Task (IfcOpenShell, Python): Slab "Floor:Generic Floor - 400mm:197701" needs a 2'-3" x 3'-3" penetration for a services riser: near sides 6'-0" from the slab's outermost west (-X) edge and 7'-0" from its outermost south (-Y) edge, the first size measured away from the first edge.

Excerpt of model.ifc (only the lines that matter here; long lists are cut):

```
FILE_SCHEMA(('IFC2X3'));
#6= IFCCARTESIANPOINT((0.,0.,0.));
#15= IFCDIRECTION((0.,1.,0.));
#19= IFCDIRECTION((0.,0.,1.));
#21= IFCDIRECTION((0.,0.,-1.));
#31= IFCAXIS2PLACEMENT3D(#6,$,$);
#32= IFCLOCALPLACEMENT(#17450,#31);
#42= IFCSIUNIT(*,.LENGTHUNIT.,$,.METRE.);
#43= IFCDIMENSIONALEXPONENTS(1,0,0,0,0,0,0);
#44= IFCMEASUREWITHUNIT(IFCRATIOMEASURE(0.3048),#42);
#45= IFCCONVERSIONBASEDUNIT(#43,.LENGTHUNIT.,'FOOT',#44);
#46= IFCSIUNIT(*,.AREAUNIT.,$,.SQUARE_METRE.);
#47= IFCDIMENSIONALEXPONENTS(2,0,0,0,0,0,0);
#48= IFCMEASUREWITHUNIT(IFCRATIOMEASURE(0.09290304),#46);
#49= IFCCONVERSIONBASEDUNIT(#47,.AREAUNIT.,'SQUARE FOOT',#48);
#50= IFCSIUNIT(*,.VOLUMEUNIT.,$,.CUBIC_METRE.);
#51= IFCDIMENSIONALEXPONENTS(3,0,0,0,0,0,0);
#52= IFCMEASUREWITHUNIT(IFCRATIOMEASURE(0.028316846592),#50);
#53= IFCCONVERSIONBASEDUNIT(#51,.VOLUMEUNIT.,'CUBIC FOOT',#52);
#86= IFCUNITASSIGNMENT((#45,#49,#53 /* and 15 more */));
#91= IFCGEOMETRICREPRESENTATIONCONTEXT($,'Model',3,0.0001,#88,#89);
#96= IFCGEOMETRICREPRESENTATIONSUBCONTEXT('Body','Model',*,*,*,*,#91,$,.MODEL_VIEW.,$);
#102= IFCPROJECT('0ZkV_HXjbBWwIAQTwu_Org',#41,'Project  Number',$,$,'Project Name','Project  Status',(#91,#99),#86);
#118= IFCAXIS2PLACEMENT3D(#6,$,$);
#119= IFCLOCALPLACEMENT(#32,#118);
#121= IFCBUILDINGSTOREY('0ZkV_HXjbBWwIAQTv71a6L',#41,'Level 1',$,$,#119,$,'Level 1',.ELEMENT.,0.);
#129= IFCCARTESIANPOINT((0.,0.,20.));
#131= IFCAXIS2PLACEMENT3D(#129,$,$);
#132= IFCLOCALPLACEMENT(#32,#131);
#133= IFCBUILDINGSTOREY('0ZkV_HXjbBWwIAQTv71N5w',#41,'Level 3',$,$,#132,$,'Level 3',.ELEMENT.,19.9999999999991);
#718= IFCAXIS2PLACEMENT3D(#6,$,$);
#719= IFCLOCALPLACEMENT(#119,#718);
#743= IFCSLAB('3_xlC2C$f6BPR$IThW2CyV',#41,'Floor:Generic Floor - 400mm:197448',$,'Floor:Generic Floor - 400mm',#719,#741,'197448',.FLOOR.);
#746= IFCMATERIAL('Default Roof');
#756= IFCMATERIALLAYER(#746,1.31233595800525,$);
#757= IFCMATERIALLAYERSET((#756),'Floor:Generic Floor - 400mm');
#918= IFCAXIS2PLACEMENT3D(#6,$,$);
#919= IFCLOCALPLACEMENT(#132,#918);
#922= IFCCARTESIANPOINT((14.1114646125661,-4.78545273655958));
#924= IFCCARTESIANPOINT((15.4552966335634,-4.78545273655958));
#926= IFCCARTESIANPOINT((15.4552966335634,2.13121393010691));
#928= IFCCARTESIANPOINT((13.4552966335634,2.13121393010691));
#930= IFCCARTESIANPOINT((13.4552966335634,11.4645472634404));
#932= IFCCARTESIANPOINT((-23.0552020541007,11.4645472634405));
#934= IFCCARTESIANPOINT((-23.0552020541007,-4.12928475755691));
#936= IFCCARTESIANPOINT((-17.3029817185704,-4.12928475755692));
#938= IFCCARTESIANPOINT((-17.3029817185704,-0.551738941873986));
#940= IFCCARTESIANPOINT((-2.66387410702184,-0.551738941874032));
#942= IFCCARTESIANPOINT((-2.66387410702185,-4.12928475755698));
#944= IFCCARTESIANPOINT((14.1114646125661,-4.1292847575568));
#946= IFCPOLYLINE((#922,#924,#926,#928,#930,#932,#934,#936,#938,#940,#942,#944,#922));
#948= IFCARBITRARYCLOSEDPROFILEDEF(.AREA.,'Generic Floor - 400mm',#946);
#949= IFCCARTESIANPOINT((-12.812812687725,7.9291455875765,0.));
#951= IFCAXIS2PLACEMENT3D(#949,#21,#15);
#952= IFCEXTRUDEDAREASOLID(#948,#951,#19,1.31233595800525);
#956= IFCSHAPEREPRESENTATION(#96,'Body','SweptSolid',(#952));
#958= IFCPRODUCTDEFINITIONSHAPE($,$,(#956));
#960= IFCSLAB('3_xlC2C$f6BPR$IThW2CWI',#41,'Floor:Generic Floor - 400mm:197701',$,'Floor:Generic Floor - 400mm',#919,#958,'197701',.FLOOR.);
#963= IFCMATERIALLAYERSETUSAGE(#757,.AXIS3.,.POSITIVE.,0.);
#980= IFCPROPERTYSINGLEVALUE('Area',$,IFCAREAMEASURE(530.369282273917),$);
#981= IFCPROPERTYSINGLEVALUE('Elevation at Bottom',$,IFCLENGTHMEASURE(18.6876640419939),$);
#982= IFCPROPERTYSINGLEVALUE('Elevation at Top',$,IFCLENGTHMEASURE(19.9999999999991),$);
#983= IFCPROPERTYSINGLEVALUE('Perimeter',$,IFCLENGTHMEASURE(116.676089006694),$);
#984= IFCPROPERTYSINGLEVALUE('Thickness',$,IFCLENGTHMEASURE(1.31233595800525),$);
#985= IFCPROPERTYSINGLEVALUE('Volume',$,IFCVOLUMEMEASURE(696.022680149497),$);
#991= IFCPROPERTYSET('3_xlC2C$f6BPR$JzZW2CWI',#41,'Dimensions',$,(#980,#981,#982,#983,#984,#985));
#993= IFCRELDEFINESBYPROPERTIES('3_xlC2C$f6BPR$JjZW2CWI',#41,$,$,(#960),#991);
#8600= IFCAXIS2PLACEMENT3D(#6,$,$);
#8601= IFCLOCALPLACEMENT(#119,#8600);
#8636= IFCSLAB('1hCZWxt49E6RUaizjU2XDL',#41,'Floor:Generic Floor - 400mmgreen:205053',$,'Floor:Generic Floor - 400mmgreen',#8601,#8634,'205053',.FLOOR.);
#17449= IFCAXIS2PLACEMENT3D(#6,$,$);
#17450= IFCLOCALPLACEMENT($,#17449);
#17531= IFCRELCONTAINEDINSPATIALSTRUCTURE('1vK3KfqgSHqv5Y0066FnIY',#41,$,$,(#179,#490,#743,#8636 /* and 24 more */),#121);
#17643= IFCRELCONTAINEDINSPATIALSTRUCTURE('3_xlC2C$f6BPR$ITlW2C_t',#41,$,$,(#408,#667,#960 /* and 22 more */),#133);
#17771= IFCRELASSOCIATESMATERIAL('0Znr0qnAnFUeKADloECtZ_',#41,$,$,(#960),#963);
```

```python
import numpy as np
import ifcopenshell
import ifcopenshell.api.feature
import ifcopenshell.api.geometry
import ifcopenshell.api.pset
import ifcopenshell.api.root
import ifcopenshell.geom
import ifcopenshell.util.element
import ifcopenshell.util.placement
import ifcopenshell.util.representation
import ifcopenshell.util.shape
import ifcopenshell.util.unit

model = ifcopenshell.open("model.ifc")
unit_scale = ifcopenshell.util.unit.calculate_unit_scale(model)
area_scale = ifcopenshell.util.unit.calculate_unit_scale(model, "AREAUNIT")
volume_scale = ifcopenshell.util.unit.calculate_unit_scale(model, "VOLUMEUNIT")
settings = ifcopenshell.geom.settings()


def volume(element):
    """Net volume in cubic metres, openings subtracted."""
    shape = ifcopenshell.geom.create_shape(settings, element)
    return ifcopenshell.util.shape.get_volume(shape.geometry)


slab = model.by_id(960)
before = volume(slab)

# Extent in the slab's own axes, in metres. The edges named are its -X and -Y sides.
slab_shape = ifcopenshell.geom.create_shape(settings, slab)
vertices = ifcopenshell.util.shape.get_vertices(slab_shape.geometry)
x_min, y_min, bottom = vertices.min(axis=0)
top = vertices[:, 2].max()

opening = ifcopenshell.api.root.create_entity(model, ifc_class="IfcOpeningElement", name="Services riser opening")
context = ifcopenshell.util.representation.get_context(model, "Model", "Body", "MODEL_VIEW")
width, depth = 0.6858, 0.9906
outline = [(0.0, 0.0), (width, 0.0), (width, depth), (0.0, depth), (0.0, 0.0)]
# Overshoot both faces by 50 mm so the cut is clean.
shape = ifcopenshell.api.geometry.add_slab_representation(
    model, context=context, depth=top - bottom + 0.1, polyline=outline
)
ifcopenshell.api.geometry.assign_representation(model, product=opening, representation=shape)

matrix = ifcopenshell.util.placement.get_local_placement(slab.ObjectPlacement)
matrix[:, 3] = matrix @ np.append(np.array([x_min + 1.8288, y_min + 2.1336, bottom - 0.05]) / unit_scale, 1.0)
ifcopenshell.api.geometry.edit_object_placement(model, product=opening, matrix=matrix, is_si=False)
ifcopenshell.api.feature.add_feature(model, feature=opening, element=slab)

after = volume(slab)

# Update the slab's stored quantities.
pset = model.by_id(ifcopenshell.util.element.get_pset(slab, "Dimensions", should_inherit=False)["id"])
ifcopenshell.api.pset.edit_pset(model, pset=pset, properties={
    "Area": model.create_entity("IfcAreaMeasure", after / (top - bottom) / area_scale),
    "Volume": model.create_entity("IfcVolumeMeasure", after / volume_scale),
})

print(f"slab volume {before:.3f} -> {after:.3f} m3")

model.write("model-out.ifc")
```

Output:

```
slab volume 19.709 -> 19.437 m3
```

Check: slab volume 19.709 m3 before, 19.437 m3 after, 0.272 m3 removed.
